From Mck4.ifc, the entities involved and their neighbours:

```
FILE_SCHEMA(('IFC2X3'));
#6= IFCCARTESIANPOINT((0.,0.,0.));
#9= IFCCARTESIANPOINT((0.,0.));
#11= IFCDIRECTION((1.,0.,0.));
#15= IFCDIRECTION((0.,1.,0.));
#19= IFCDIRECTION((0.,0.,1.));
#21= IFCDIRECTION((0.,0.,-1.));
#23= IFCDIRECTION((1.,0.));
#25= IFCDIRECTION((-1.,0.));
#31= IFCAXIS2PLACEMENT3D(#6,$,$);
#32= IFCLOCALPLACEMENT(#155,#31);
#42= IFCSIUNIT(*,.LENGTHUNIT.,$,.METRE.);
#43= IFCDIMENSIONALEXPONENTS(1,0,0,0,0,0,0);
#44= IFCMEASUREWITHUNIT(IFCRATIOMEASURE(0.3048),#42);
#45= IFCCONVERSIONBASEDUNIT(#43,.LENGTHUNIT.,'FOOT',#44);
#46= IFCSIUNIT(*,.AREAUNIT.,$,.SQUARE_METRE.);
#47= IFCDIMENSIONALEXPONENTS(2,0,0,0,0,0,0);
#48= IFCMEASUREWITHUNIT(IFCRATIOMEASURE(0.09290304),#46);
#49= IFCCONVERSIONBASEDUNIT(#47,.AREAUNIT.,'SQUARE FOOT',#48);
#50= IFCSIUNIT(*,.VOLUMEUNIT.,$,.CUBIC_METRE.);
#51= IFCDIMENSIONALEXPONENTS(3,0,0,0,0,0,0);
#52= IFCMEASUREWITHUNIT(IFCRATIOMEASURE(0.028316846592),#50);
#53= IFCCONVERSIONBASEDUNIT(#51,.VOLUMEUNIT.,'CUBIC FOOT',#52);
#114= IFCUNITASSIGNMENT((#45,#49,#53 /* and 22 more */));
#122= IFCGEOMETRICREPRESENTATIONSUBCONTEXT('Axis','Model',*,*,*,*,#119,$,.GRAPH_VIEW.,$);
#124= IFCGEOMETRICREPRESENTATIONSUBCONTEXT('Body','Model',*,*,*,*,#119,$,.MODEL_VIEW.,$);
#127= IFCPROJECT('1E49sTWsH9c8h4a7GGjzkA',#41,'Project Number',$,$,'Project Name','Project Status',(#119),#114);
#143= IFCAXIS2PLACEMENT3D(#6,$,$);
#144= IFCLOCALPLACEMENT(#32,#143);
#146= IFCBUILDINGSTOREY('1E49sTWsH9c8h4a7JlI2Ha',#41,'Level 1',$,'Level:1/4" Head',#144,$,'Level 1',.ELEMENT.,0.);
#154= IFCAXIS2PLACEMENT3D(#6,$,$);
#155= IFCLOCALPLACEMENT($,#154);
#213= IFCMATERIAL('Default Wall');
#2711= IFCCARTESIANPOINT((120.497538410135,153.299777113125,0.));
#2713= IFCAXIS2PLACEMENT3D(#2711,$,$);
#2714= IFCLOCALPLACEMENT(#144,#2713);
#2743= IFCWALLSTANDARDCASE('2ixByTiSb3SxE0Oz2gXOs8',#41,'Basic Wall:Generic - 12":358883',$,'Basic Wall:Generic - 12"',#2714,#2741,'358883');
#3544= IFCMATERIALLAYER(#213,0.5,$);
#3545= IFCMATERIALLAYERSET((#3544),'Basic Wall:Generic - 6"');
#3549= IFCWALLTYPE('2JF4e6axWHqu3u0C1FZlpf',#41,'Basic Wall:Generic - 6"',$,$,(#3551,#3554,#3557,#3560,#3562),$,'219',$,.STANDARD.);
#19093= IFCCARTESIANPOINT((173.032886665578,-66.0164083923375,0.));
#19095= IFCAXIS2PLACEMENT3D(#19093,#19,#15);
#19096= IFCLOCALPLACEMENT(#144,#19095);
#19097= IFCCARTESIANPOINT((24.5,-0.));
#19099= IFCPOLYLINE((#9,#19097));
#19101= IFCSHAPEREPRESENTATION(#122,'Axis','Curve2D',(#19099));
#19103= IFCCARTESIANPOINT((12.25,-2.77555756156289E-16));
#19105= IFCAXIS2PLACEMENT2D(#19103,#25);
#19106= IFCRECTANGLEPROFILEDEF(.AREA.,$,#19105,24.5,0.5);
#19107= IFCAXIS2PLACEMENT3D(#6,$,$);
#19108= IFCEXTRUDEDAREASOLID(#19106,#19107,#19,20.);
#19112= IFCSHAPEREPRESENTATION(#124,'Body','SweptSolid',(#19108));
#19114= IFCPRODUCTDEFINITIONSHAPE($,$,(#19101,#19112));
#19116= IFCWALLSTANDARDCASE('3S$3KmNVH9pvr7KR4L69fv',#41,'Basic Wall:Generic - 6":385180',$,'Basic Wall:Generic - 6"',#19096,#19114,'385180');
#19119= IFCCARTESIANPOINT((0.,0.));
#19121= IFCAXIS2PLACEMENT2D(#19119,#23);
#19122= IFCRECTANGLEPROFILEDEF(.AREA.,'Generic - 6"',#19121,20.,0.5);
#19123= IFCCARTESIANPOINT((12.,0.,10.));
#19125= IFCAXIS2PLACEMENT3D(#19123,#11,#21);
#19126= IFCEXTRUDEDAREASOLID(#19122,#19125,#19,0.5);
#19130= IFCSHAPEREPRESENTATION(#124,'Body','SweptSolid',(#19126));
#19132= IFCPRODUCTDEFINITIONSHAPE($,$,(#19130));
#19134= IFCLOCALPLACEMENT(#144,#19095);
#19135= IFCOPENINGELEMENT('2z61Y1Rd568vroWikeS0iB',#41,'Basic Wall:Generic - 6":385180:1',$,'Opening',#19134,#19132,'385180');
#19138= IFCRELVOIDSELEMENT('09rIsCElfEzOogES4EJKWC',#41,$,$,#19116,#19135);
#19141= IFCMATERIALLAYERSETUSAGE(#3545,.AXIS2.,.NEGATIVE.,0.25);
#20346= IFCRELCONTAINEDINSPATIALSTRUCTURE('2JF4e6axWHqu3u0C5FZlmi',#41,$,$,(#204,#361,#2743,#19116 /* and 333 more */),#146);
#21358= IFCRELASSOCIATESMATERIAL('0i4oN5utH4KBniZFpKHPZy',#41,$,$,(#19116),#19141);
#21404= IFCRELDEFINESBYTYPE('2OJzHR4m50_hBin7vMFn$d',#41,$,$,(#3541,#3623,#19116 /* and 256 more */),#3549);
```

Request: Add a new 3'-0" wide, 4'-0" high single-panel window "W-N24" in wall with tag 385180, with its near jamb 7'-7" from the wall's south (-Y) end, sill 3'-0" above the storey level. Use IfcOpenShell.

```python
import numpy as np
import ifcopenshell
import ifcopenshell.api.feature
import ifcopenshell.api.geometry
import ifcopenshell.api.root
import ifcopenshell.api.spatial
import ifcopenshell.api.type
import ifcopenshell.geom
import ifcopenshell.util.element
import ifcopenshell.util.placement
import ifcopenshell.util.representation
import ifcopenshell.util.shape
import ifcopenshell.util.unit

model = ifcopenshell.open("Mck4.ifc")
unit_scale = ifcopenshell.util.unit.calculate_unit_scale(model)
settings = ifcopenshell.geom.settings()


def volume(element):
    """Net volume in cubic metres, openings subtracted."""
    shape = ifcopenshell.geom.create_shape(settings, element)
    return ifcopenshell.util.shape.get_volume(shape.geometry)


wall = model.by_id(19116)
storey = ifcopenshell.util.element.get_container(wall, ifc_class="IfcBuildingStorey")
context = ifcopenshell.util.representation.get_context(model, "Model", "Body", "MODEL_VIEW")
before = volume(wall)

width, height, from_end, sill = 0.9144, 1.2192, 2.3114, 0.9144  # metres

# The wall runs along its own X axis, and the end named is its -X end.
wall_shape = ifcopenshell.geom.create_shape(settings, wall)
x, y, z = ifcopenshell.util.shape.get_vertices(wall_shape.geometry).T
start = x.min() + from_end
face, thickness = float(y.min()), float(y.max() - y.min())
wall_matrix = ifcopenshell.util.placement.get_local_placement(wall.ObjectPlacement)
level = ifcopenshell.util.placement.get_local_placement(storey.ObjectPlacement)[2, 3]


def in_wall(x, y):
    """Placement at x, y metres in the wall's axes, at sill height."""
    matrix = wall_matrix.copy()
    matrix[:, 3] = wall_matrix @ np.array([x / unit_scale, y / unit_scale, 0.0, 1.0])
    matrix[2, 3] = level + sill / unit_scale
    return matrix


# Opening: a box that overshoots both wall faces by 50 mm.
opening = ifcopenshell.api.root.create_entity(model, ifc_class="IfcOpeningElement")
box = ifcopenshell.api.geometry.add_wall_representation(
    model, context=context, length=width, height=height, thickness=thickness + 0.1
)
ifcopenshell.api.geometry.assign_representation(model, product=opening, representation=box)
ifcopenshell.api.geometry.edit_object_placement(model, product=opening, matrix=in_wall(start, face - 0.05), is_si=False)
ifcopenshell.api.feature.add_feature(model, feature=opening, element=wall)

window = ifcopenshell.api.root.create_entity(model, ifc_class="IfcWindow", name="W-N24")
window.OverallWidth, window.OverallHeight = width / unit_scale, height / unit_scale
body = ifcopenshell.api.geometry.add_window_representation(
    model,
    context=context,
    overall_width=window.OverallWidth,
    overall_height=window.OverallHeight,
    partition_type="SINGLE_PANEL",
)
ifcopenshell.api.geometry.assign_representation(model, product=window, representation=body)
ifcopenshell.api.spatial.assign_container(model, products=[window], relating_structure=storey)
fills = ifcopenshell.api.feature.add_filling(model, opening=opening, element=window)
fills.OwnerHistory = window.OwnerHistory  # required in IFC2X3

# IFC2X3 keeps the operation on the window style.
style = ifcopenshell.api.root.create_entity(model, ifc_class="IfcWindowStyle", name="W-N24")
style.OperationType, style.ConstructionType = "SINGLE_PANEL", "NOTDEFINED"
style.ParameterTakesPrecedence = style.Sizeable = False
ifcopenshell.api.type.assign_type(model, related_objects=[window], relating_type=style)

# Centre the window in the wall's thickness.
ifcopenshell.api.geometry.edit_object_placement(model, product=window, matrix=in_wall(start, face), is_si=False)
window_shape = ifcopenshell.geom.create_shape(settings, window)
depth = ifcopenshell.util.shape.get_vertices(window_shape.geometry)[:, 1]
offset = face + thickness / 2 - (depth.min() + depth.max()) / 2
ifcopenshell.api.geometry.edit_object_placement(model, product=window, matrix=in_wall(start, offset), is_si=False)

after = volume(wall)

print(f"wall volume {before:.3f} -> {after:.3f} m3")

model.write("Mck4-out.ifc")
```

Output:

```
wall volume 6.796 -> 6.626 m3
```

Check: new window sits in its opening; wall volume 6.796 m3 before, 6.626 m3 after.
